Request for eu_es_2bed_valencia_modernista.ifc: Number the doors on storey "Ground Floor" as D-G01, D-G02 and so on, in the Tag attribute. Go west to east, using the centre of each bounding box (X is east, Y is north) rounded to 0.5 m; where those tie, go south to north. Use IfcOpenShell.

First a look at what the model holds.

```python
import ifcopenshell
import ifcopenshell.util.element
import ifcopenshell.util.placement

model = ifcopenshell.open("eu_es_2bed_valencia_modernista.ifc")
print(model.schema)
storey = next(s for s in model.by_type("IfcBuildingStorey") if s.Name == "Ground Floor")
doors = [e for e in ifcopenshell.util.element.get_decomposition(storey) if e.is_a("IfcDoor")]
for e in sorted(doors, key=lambda e: e.id()):
    origin = ifcopenshell.util.placement.get_local_placement(e.ObjectPlacement)[:3, 3]
    print(e.id(), e.Tag, e.Name, origin.round(2) + 0.0, sep=" | ")
```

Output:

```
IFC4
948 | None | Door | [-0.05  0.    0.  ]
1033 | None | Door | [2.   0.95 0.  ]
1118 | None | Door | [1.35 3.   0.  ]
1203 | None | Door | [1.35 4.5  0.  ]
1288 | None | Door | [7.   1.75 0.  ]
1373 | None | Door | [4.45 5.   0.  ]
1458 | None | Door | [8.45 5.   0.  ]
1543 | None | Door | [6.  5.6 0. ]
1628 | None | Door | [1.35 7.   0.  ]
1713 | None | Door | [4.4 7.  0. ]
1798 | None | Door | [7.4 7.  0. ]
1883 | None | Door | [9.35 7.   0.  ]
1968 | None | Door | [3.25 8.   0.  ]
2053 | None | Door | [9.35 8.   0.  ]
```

```python
import ifcopenshell
import ifcopenshell.geom
import ifcopenshell.util.element
import ifcopenshell.util.shape

model = ifcopenshell.open("eu_es_2bed_valencia_modernista.ifc")
settings = ifcopenshell.geom.settings()
settings.set("use-world-coords", True)


def centre(element):
    shape = ifcopenshell.geom.create_shape(settings, element)
    return ifcopenshell.util.shape.get_bbox_centroid(shape.geometry)


storey = next(s for s in model.by_type("IfcBuildingStorey") if s.Name == "Ground Floor")
doors = [e for e in ifcopenshell.util.element.get_decomposition(storey) if e.is_a("IfcDoor")]

# Insertion points can sit at a corner or the storey origin, so sort by the geometry (in metres).
centres = {e: centre(e) for e in doors}
doors.sort(key=lambda e: (round(centres[e][0] / 0.5), centres[e][1]))

for i, e in enumerate(doors, start=1):
    number = f"D-G{i:02d}"
    e.Tag = number
    print(e.id(), number)

model.write("eu_es_2bed_valencia_modernista_updated.ifc")
```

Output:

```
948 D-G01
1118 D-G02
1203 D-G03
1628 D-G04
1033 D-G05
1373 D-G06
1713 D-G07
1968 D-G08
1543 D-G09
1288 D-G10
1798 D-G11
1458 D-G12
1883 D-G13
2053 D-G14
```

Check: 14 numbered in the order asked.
